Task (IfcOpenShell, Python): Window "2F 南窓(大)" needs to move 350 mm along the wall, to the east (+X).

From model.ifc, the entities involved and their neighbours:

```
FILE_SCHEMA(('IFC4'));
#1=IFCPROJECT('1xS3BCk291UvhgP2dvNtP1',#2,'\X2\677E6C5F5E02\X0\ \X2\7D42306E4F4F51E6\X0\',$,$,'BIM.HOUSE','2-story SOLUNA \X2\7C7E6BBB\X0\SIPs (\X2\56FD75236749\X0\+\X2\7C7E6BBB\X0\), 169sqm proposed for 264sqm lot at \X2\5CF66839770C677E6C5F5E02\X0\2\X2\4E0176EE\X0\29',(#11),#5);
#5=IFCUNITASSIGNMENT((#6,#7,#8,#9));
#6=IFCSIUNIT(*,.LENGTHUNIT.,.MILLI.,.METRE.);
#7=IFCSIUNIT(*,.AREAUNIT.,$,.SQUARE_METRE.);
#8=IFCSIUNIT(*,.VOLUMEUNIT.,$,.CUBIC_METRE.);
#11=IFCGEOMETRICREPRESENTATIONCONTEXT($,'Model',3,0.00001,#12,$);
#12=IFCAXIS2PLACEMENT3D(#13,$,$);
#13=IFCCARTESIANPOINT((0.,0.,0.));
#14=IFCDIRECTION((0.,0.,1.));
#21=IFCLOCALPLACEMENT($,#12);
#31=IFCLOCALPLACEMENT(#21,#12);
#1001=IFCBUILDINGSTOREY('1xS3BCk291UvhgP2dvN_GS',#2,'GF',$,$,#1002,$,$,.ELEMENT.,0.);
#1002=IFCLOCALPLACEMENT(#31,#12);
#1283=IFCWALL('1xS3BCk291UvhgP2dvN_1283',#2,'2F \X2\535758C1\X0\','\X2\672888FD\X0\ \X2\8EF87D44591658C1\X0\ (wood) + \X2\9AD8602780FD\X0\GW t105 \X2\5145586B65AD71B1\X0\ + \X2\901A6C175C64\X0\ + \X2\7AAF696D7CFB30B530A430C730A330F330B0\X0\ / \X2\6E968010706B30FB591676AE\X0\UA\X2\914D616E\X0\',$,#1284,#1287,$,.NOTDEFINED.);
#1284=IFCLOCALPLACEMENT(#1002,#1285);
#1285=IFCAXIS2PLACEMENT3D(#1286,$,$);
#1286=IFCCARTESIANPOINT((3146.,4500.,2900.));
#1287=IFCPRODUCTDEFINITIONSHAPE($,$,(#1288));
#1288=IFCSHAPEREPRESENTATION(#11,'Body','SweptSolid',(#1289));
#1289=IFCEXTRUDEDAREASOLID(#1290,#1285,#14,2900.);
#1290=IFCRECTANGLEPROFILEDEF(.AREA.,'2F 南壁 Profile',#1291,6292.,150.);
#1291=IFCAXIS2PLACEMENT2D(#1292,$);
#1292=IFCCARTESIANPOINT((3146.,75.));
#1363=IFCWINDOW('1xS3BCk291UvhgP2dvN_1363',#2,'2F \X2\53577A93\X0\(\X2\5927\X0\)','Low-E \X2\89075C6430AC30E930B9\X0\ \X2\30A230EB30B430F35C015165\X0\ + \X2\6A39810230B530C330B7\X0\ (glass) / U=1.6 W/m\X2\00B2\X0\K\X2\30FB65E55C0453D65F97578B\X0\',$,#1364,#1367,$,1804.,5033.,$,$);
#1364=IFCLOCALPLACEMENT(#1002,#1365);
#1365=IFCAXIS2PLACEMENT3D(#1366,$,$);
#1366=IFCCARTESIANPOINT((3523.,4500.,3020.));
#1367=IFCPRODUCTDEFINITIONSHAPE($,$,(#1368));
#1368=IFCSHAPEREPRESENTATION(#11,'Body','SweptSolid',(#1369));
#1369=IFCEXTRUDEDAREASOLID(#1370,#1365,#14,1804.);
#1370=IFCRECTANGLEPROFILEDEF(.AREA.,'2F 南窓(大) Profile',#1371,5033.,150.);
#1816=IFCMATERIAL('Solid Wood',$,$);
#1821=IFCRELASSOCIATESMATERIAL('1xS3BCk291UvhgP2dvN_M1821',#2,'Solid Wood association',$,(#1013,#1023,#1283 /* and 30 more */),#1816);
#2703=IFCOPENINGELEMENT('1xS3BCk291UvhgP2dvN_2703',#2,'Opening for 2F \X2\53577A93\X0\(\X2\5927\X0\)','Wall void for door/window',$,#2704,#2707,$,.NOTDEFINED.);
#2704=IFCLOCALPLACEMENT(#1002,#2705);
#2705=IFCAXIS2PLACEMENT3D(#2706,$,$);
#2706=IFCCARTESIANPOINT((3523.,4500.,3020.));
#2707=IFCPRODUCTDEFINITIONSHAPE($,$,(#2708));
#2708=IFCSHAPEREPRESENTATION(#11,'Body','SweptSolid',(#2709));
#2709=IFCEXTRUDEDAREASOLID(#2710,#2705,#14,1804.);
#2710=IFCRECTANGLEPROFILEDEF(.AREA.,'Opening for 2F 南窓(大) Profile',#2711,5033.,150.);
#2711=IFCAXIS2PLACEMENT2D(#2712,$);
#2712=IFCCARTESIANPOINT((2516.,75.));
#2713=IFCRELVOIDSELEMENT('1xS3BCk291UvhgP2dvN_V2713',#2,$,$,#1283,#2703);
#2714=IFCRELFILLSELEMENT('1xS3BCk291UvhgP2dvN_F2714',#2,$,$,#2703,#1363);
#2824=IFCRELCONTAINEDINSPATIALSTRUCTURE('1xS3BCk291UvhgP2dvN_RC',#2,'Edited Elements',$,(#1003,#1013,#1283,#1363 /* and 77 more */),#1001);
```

```python
import ifcopenshell
import ifcopenshell.api.geometry
import ifcopenshell.util.placement

model = ifcopenshell.open("model.ifc")

window = model.by_guid("1xS3BCk291UvhgP2dvN_1363")
opening = window.FillsVoids[0].RelatingOpeningElement
wall = opening.VoidsElements[0].RelatingBuildingElement

wall_matrix = ifcopenshell.util.placement.get_local_placement(wall.ObjectPlacement)
shift = wall_matrix[:3, 0] * 350.0
before = ifcopenshell.util.placement.get_local_placement(window.ObjectPlacement)[:3, 3].copy()

# The window is not placed relative to its opening, so move both.
for product in (opening, window):
    matrix = ifcopenshell.util.placement.get_local_placement(product.ObjectPlacement)
    matrix[:3, 3] += shift
    ifcopenshell.api.geometry.edit_object_placement(model, product=product, matrix=matrix, is_si=False)

after = ifcopenshell.util.placement.get_local_placement(window.ObjectPlacement)[:3, 3]
print("window moved by", (after - before).round(3) + 0.0)

model.write("model_v2.ifc")
```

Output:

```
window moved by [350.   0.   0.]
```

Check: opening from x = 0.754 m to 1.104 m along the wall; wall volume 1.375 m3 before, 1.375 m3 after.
